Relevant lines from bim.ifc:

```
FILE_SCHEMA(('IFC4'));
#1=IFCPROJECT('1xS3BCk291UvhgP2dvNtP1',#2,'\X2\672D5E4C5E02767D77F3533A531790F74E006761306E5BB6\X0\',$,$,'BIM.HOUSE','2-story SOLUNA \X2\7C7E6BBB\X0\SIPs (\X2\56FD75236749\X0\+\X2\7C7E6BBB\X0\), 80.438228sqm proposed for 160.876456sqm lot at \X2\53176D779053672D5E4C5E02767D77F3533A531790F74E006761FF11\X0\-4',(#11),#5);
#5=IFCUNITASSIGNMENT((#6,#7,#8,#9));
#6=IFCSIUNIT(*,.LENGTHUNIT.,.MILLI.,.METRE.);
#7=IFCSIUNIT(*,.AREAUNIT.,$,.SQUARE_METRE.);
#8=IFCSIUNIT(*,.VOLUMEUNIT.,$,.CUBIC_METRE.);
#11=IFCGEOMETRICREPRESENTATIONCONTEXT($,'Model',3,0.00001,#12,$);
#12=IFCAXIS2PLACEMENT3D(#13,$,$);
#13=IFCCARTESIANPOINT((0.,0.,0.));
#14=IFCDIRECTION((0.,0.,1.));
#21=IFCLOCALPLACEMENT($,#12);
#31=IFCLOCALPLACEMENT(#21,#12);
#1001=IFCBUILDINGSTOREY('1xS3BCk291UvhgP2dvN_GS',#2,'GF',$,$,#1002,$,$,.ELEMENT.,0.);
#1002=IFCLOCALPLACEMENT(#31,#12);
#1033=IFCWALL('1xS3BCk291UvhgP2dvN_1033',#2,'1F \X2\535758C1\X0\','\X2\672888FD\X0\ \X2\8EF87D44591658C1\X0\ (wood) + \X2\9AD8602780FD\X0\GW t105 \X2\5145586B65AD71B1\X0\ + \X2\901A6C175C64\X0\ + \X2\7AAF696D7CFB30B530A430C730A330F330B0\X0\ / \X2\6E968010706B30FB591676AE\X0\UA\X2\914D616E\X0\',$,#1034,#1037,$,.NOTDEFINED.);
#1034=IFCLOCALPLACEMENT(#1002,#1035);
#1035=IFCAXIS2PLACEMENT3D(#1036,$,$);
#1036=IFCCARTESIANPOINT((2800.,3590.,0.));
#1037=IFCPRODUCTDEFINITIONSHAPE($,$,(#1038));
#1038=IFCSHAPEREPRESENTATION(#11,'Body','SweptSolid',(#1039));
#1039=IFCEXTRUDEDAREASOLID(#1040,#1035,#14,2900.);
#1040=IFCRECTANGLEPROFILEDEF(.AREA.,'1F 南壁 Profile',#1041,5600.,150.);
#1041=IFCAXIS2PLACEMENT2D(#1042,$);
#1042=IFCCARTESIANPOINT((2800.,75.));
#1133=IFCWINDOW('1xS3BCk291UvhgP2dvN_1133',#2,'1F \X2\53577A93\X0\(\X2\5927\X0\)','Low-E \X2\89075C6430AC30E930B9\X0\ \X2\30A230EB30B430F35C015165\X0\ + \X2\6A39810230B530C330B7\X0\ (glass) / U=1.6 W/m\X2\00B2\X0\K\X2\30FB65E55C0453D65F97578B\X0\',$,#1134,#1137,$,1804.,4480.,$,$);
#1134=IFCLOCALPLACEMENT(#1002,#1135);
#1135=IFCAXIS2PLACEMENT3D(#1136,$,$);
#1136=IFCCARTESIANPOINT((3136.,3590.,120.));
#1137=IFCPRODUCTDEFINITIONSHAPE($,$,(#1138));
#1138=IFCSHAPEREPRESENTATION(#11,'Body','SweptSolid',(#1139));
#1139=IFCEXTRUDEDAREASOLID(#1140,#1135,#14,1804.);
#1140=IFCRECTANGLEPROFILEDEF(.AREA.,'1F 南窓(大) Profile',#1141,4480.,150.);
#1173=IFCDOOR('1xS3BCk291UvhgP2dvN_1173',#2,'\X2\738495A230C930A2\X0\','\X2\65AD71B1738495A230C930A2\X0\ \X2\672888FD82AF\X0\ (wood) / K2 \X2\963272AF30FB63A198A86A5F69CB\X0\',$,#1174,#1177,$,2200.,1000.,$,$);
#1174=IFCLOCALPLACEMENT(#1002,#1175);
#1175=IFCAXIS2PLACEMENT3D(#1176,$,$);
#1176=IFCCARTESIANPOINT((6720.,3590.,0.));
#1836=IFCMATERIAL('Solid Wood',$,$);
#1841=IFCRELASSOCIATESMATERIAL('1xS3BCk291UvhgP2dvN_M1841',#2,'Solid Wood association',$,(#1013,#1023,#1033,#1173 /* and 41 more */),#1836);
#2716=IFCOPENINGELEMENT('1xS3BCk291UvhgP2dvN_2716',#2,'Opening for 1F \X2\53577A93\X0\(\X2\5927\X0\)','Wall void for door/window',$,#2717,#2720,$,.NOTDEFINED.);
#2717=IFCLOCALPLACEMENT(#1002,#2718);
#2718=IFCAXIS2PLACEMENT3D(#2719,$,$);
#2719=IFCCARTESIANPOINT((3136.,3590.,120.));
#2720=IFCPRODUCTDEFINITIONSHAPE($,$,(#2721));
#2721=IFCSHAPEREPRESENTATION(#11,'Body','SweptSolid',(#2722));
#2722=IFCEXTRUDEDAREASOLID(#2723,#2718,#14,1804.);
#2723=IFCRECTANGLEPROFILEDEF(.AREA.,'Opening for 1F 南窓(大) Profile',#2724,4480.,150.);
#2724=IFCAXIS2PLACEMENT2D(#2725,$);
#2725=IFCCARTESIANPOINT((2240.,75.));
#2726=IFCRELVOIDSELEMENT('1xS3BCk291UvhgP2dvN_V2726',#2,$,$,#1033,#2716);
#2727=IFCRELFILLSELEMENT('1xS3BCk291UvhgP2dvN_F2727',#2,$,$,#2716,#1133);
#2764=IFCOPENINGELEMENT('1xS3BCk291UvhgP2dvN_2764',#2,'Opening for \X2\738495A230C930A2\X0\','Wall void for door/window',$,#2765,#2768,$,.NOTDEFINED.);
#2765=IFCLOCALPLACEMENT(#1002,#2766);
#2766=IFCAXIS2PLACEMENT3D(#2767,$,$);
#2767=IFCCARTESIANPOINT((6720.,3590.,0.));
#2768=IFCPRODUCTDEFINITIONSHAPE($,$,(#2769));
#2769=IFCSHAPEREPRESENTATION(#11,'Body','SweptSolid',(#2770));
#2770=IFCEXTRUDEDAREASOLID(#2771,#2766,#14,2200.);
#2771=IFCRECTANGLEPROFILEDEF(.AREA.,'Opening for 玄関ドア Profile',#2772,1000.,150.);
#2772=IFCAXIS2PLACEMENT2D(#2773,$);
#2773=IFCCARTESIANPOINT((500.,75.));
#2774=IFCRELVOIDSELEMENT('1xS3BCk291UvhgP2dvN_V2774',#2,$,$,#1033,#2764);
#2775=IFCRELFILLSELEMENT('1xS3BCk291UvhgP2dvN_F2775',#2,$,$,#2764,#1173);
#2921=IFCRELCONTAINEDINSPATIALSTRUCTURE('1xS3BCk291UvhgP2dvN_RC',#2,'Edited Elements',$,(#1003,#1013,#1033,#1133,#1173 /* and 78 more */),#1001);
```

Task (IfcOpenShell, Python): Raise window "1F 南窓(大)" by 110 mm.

```python
import numpy as np
import ifcopenshell
import ifcopenshell.api.geometry
import ifcopenshell.util.placement
import ifcopenshell.util.unit

model = ifcopenshell.open("bim.ifc")
unit_scale = ifcopenshell.util.unit.calculate_unit_scale(model)

window = model.by_id(1133)
opening = window.FillsVoids[0].RelatingOpeningElement
dz = 0.11 / unit_scale

shift = np.array([0.0, 0.0, dz])
# The window is not placed relative to its opening, so move both.
for product in (opening, window):
    matrix = ifcopenshell.util.placement.get_local_placement(product.ObjectPlacement)
    matrix[:3, 3] += shift
    ifcopenshell.api.geometry.edit_object_placement(model, product=product, matrix=matrix, is_si=False)

print(f"moved by {dz * unit_scale:+.3f} m")

model.write("bim_edited.ifc")
```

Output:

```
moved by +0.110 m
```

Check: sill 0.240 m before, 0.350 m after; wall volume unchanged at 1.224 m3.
